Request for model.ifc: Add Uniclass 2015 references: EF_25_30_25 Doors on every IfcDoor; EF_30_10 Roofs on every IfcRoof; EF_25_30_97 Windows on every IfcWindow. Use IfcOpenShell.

First a look at what the model holds.

```python
import ifcopenshell

model = ifcopenshell.open("model.ifc")
print(model.schema)
print("classifications:", [c.Name for c in model.by_type("IfcClassification")])
for ifc_class in ("IfcDoor", "IfcRoof", "IfcStair", "IfcWall", "IfcWindow"):
    print(ifc_class, len(model.by_type(ifc_class)))
```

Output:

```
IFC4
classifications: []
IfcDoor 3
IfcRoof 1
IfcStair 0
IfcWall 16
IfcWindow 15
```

```python
import ifcopenshell
import ifcopenshell.api.classification

model = ifcopenshell.open("model.ifc")

system = ifcopenshell.api.classification.add_classification(model, classification="Uniclass 2015")

codes = {
    "IfcDoor": ("EF_25_30_25", "Doors"),
    "IfcRoof": ("EF_30_10", "Roofs"),
    "IfcWindow": ("EF_25_30_97", "Windows"),
}
for ifc_class, (code, name) in codes.items():
    products = model.by_type(ifc_class)
    ifcopenshell.api.classification.add_reference(
        model, products=products, classification=system, identification=code, name=name
    )
    print(code, len(products))

model.write("model-out.ifc")
```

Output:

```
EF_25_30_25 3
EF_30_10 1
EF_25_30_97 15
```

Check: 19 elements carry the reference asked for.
